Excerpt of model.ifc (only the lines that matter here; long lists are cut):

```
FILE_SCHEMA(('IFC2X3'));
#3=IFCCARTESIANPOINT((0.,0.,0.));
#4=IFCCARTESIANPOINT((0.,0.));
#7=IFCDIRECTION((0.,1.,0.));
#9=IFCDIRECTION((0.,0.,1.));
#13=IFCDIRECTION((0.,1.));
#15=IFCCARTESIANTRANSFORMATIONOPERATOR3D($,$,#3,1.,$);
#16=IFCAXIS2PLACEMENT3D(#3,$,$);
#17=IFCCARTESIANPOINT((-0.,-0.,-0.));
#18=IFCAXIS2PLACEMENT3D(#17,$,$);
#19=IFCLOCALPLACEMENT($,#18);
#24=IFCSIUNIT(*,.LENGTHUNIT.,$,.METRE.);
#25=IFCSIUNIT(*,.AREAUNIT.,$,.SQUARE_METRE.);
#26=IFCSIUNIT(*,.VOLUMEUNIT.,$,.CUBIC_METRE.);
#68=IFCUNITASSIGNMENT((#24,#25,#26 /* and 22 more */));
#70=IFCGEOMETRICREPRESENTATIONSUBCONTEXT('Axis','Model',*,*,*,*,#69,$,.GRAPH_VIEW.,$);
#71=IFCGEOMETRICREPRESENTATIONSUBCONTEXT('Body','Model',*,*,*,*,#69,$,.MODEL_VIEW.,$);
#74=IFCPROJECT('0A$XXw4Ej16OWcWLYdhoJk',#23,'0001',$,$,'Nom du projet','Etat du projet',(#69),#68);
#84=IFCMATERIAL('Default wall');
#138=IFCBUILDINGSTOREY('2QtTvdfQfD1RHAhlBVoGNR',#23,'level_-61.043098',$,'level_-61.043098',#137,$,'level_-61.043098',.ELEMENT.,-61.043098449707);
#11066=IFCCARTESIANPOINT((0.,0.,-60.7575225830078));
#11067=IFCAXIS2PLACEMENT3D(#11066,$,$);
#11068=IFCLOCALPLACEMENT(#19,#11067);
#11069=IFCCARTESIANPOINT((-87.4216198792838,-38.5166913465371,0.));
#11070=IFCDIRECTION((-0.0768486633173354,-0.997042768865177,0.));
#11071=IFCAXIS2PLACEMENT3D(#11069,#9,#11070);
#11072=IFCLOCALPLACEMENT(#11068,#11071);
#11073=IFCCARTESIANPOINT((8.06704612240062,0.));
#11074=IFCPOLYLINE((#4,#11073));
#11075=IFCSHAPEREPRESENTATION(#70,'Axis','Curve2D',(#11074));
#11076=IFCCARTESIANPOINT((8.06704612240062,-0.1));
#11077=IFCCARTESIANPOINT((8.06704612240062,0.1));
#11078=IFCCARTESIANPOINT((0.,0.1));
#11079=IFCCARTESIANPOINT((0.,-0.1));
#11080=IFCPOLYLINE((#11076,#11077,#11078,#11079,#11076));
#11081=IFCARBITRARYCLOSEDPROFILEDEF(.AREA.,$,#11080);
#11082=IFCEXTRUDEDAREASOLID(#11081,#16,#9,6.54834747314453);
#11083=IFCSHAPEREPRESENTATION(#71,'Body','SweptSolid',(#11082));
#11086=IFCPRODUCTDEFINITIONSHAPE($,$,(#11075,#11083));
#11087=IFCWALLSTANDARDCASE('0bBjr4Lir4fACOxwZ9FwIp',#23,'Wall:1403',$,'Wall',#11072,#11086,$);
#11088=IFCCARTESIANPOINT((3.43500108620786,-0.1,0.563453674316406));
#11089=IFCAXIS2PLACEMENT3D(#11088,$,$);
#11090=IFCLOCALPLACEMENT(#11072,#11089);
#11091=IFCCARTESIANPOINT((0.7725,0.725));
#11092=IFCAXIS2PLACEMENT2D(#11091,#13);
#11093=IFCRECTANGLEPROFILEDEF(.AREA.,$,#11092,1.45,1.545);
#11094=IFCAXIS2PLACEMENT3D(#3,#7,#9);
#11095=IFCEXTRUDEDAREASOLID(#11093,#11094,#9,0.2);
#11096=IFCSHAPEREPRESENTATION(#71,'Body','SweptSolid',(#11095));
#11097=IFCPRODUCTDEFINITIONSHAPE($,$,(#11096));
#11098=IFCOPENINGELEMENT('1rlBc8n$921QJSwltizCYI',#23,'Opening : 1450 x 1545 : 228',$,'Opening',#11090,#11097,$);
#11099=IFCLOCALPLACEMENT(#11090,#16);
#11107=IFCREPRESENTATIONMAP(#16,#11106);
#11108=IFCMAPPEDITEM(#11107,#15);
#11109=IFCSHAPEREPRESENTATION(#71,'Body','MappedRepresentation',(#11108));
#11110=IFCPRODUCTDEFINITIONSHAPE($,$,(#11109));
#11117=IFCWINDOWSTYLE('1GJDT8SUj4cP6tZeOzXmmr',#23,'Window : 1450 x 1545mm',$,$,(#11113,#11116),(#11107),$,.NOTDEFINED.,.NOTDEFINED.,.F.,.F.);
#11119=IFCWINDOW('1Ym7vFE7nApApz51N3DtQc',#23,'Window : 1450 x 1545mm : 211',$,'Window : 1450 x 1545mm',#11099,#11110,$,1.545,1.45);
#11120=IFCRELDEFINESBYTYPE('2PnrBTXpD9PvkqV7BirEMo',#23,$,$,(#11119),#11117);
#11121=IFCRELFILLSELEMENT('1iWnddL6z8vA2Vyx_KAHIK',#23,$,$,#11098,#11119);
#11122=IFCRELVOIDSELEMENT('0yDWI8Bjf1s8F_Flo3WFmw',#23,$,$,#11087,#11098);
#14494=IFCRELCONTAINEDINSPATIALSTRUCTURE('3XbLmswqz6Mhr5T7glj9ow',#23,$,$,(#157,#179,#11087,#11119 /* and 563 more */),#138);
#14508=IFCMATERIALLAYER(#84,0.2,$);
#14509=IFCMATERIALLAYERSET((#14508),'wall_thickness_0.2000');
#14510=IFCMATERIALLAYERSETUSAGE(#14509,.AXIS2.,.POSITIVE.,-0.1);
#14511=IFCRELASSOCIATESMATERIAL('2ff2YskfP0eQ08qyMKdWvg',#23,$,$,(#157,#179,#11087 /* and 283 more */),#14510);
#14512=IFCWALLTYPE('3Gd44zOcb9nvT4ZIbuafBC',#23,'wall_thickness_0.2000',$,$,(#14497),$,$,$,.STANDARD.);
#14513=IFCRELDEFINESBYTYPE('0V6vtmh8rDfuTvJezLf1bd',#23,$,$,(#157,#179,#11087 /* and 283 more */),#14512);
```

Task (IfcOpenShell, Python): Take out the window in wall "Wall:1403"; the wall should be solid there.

```python
import ifcopenshell
import ifcopenshell.api.feature
import ifcopenshell.api.root
import ifcopenshell.geom
import ifcopenshell.util.shape

model = ifcopenshell.open("model.ifc")
settings = ifcopenshell.geom.settings()


def volume(element):
    """Net volume in cubic metres, openings subtracted."""
    shape = ifcopenshell.geom.create_shape(settings, element)
    return ifcopenshell.util.shape.get_volume(shape.geometry)


window = model.by_guid("1Ym7vFE7nApApz51N3DtQc")
opening = window.FillsVoids[0].RelatingOpeningElement
wall = opening.VoidsElements[0].RelatingBuildingElement
before = volume(wall)

ifcopenshell.api.root.remove_product(model, product=window)
ifcopenshell.api.feature.remove_feature(model, feature=opening)

after = volume(wall)

print(f"wall volume {before:.3f} -> {after:.3f} m3")

model.write("model-out.ifc")
```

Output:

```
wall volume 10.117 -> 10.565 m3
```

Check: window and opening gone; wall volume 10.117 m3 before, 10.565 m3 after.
